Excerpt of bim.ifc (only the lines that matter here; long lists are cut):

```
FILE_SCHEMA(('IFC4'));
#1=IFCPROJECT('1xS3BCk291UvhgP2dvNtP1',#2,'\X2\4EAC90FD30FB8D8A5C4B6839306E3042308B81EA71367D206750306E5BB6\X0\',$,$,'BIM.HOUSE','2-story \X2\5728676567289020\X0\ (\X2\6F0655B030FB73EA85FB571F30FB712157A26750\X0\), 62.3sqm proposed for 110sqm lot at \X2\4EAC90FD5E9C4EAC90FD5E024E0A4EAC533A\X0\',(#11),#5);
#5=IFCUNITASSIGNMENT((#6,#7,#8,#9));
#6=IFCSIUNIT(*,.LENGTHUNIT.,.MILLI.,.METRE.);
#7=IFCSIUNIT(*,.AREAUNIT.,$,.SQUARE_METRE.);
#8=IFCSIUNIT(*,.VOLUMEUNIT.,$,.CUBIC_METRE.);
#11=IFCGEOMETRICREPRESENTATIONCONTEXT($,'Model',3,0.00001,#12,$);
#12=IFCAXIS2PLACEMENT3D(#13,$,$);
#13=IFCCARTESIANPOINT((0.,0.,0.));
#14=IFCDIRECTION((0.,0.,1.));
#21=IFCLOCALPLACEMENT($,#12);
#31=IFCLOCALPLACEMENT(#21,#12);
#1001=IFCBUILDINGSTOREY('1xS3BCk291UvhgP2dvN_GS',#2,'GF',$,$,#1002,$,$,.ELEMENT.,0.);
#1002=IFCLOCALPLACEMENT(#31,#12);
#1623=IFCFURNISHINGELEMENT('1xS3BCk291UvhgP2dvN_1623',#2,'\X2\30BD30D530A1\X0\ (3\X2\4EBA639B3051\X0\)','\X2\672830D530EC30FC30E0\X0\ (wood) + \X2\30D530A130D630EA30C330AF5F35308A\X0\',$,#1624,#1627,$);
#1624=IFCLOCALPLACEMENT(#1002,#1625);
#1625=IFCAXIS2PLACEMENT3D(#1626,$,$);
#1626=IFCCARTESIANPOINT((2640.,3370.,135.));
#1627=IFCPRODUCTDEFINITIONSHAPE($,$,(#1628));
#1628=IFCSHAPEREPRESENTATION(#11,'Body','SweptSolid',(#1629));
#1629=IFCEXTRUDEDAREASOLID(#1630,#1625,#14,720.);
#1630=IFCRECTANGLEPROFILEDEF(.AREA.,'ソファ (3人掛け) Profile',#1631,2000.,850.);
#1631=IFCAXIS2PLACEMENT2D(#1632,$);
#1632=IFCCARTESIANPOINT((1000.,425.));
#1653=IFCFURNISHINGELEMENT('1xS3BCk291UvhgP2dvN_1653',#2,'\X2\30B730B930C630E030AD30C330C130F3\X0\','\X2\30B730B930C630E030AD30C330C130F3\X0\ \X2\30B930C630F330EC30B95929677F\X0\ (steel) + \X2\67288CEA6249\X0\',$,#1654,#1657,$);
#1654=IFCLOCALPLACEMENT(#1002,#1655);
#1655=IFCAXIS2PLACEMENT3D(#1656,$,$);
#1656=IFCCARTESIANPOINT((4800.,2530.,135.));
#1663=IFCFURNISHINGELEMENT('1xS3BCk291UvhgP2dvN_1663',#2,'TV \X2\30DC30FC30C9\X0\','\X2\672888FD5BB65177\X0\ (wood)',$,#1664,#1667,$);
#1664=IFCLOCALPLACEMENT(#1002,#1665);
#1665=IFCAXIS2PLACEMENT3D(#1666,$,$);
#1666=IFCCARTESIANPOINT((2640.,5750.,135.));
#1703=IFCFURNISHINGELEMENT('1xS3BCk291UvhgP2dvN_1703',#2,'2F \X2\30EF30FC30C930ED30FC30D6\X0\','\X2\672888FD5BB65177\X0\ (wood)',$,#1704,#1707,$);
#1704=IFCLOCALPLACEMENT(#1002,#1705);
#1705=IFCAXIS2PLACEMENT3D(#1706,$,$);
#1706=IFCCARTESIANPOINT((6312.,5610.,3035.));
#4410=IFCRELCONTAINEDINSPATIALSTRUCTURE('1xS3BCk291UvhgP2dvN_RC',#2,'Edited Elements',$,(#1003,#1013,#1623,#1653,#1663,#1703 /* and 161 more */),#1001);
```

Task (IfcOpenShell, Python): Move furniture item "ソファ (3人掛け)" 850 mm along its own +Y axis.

```python
import ifcopenshell
import ifcopenshell.api.geometry
import ifcopenshell.util.placement

model = ifcopenshell.open("bim.ifc")

item = model.by_id(1623)
matrix = ifcopenshell.util.placement.get_local_placement(item.ObjectPlacement)
matrix[:3, 3] += matrix[:3, 1] * 850.0
ifcopenshell.api.geometry.edit_object_placement(model, product=item, matrix=matrix, is_si=False)

print(ifcopenshell.util.placement.get_local_placement(item.ObjectPlacement).round(3) + 0.0)

model.write("bim_edited.ifc")
```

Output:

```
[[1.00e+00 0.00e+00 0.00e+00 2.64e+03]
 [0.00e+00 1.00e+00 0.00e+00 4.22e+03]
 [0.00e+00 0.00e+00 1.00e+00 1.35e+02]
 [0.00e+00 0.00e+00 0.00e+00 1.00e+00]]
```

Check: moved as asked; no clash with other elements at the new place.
